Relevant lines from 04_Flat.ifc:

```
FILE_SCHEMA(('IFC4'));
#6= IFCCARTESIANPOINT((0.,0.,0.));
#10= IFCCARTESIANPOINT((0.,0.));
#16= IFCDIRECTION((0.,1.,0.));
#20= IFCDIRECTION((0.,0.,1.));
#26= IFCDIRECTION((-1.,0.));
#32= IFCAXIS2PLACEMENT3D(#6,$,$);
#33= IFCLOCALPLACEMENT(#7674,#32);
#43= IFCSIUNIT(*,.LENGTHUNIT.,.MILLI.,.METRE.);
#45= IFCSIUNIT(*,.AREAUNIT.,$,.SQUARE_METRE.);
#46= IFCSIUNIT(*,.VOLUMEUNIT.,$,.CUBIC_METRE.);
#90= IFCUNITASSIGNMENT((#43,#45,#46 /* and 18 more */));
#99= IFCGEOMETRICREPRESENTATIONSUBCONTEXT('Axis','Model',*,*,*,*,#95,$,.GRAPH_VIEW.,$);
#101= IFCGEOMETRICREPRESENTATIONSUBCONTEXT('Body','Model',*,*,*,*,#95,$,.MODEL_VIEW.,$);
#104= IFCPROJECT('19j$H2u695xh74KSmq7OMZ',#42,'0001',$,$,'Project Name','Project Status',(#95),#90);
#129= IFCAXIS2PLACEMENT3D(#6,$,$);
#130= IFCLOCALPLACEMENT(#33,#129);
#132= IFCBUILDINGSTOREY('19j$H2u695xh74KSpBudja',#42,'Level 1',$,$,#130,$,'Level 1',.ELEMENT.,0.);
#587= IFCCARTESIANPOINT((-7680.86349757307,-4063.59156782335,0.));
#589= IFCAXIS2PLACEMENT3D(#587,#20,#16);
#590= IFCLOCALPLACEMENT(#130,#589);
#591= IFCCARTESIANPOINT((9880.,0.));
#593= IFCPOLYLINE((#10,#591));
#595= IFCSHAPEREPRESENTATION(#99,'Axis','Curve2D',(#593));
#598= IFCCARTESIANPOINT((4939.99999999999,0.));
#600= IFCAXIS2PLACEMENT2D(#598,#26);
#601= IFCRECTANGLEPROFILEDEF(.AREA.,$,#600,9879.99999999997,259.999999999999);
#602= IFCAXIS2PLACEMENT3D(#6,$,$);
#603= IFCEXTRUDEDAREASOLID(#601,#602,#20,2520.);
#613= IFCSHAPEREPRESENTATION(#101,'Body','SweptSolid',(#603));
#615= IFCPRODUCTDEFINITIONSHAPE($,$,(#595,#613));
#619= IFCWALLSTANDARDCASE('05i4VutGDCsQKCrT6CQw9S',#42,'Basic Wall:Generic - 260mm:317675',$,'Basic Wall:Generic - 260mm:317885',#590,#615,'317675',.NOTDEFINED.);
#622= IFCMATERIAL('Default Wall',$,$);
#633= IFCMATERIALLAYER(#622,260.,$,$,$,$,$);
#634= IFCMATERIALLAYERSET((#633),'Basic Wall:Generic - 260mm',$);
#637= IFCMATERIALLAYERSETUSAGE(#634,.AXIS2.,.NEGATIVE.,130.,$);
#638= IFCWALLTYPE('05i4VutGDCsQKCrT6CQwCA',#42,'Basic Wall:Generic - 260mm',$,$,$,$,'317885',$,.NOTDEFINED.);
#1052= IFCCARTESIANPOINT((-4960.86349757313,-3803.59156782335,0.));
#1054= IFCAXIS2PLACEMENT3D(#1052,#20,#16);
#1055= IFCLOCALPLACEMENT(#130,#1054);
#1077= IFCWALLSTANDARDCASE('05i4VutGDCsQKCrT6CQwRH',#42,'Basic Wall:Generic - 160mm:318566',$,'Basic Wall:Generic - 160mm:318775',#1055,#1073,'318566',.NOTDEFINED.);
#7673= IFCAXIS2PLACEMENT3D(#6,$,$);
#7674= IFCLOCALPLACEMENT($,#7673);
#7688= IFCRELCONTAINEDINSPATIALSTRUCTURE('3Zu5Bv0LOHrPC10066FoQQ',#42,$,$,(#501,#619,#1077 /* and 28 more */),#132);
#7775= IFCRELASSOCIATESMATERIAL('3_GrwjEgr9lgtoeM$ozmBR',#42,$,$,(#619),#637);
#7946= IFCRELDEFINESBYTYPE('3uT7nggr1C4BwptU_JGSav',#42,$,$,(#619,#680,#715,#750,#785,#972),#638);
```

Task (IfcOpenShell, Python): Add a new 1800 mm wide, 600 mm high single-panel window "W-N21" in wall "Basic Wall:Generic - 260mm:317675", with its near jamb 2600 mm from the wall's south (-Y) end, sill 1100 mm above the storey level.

```python
import numpy as np
import ifcopenshell
import ifcopenshell.api.feature
import ifcopenshell.api.geometry
import ifcopenshell.api.root
import ifcopenshell.api.spatial
import ifcopenshell.geom
import ifcopenshell.util.element
import ifcopenshell.util.placement
import ifcopenshell.util.representation
import ifcopenshell.util.shape
import ifcopenshell.util.unit

model = ifcopenshell.open("04_Flat.ifc")
unit_scale = ifcopenshell.util.unit.calculate_unit_scale(model)
settings = ifcopenshell.geom.settings()


def volume(element):
    """Net volume in cubic metres, openings subtracted."""
    shape = ifcopenshell.geom.create_shape(settings, element)
    return ifcopenshell.util.shape.get_volume(shape.geometry)


wall = model.by_guid("05i4VutGDCsQKCrT6CQw9S")
storey = ifcopenshell.util.element.get_container(wall, ifc_class="IfcBuildingStorey")
context = ifcopenshell.util.representation.get_context(model, "Model", "Body", "MODEL_VIEW")
before = volume(wall)

width, height, from_end, sill = 1.8, 0.6, 2.6, 1.1  # metres

# The wall runs along its own X axis, and the end named is its -X end.
wall_shape = ifcopenshell.geom.create_shape(settings, wall)
x, y, z = ifcopenshell.util.shape.get_vertices(wall_shape.geometry).T
start = x.min() + from_end
face, thickness = float(y.min()), float(y.max() - y.min())
wall_matrix = ifcopenshell.util.placement.get_local_placement(wall.ObjectPlacement)
level = ifcopenshell.util.placement.get_local_placement(storey.ObjectPlacement)[2, 3]


def in_wall(x, y):
    """Placement at x, y metres in the wall's axes, at sill height."""
    matrix = wall_matrix.copy()
    matrix[:, 3] = wall_matrix @ np.array([x / unit_scale, y / unit_scale, 0.0, 1.0])
    matrix[2, 3] = level + sill / unit_scale
    return matrix


# Opening: a box that overshoots both wall faces by 50 mm.
opening = ifcopenshell.api.root.create_entity(model, ifc_class="IfcOpeningElement", predefined_type="OPENING")
box = ifcopenshell.api.geometry.add_wall_representation(
    model, context=context, length=width, height=height, thickness=thickness + 0.1
)
ifcopenshell.api.geometry.assign_representation(model, product=opening, representation=box)
ifcopenshell.api.geometry.edit_object_placement(model, product=opening, matrix=in_wall(start, face - 0.05), is_si=False)
ifcopenshell.api.feature.add_feature(model, feature=opening, element=wall)

window = ifcopenshell.api.root.create_entity(model, ifc_class="IfcWindow", name="W-N21", predefined_type="WINDOW")
window.OverallWidth, window.OverallHeight = width / unit_scale, height / unit_scale
window.PartitioningType = "SINGLE_PANEL"
body = ifcopenshell.api.geometry.add_window_representation(
    model,
    context=context,
    overall_width=window.OverallWidth,
    overall_height=window.OverallHeight,
    partition_type="SINGLE_PANEL",
)
ifcopenshell.api.geometry.assign_representation(model, product=window, representation=body)
ifcopenshell.api.spatial.assign_container(model, products=[window], relating_structure=storey)
ifcopenshell.api.feature.add_filling(model, opening=opening, element=window)

# Centre the window in the wall's thickness.
ifcopenshell.api.geometry.edit_object_placement(model, product=window, matrix=in_wall(start, face), is_si=False)
window_shape = ifcopenshell.geom.create_shape(settings, window)
depth = ifcopenshell.util.shape.get_vertices(window_shape.geometry)[:, 1]
offset = face + thickness / 2 - (depth.min() + depth.max()) / 2
ifcopenshell.api.geometry.edit_object_placement(model, product=window, matrix=in_wall(start, offset), is_si=False)

after = volume(wall)

print(f"wall volume {before:.3f} -> {after:.3f} m3")

model.write("04_Flat_edited.ifc")
```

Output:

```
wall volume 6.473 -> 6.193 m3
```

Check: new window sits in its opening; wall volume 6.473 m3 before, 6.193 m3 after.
